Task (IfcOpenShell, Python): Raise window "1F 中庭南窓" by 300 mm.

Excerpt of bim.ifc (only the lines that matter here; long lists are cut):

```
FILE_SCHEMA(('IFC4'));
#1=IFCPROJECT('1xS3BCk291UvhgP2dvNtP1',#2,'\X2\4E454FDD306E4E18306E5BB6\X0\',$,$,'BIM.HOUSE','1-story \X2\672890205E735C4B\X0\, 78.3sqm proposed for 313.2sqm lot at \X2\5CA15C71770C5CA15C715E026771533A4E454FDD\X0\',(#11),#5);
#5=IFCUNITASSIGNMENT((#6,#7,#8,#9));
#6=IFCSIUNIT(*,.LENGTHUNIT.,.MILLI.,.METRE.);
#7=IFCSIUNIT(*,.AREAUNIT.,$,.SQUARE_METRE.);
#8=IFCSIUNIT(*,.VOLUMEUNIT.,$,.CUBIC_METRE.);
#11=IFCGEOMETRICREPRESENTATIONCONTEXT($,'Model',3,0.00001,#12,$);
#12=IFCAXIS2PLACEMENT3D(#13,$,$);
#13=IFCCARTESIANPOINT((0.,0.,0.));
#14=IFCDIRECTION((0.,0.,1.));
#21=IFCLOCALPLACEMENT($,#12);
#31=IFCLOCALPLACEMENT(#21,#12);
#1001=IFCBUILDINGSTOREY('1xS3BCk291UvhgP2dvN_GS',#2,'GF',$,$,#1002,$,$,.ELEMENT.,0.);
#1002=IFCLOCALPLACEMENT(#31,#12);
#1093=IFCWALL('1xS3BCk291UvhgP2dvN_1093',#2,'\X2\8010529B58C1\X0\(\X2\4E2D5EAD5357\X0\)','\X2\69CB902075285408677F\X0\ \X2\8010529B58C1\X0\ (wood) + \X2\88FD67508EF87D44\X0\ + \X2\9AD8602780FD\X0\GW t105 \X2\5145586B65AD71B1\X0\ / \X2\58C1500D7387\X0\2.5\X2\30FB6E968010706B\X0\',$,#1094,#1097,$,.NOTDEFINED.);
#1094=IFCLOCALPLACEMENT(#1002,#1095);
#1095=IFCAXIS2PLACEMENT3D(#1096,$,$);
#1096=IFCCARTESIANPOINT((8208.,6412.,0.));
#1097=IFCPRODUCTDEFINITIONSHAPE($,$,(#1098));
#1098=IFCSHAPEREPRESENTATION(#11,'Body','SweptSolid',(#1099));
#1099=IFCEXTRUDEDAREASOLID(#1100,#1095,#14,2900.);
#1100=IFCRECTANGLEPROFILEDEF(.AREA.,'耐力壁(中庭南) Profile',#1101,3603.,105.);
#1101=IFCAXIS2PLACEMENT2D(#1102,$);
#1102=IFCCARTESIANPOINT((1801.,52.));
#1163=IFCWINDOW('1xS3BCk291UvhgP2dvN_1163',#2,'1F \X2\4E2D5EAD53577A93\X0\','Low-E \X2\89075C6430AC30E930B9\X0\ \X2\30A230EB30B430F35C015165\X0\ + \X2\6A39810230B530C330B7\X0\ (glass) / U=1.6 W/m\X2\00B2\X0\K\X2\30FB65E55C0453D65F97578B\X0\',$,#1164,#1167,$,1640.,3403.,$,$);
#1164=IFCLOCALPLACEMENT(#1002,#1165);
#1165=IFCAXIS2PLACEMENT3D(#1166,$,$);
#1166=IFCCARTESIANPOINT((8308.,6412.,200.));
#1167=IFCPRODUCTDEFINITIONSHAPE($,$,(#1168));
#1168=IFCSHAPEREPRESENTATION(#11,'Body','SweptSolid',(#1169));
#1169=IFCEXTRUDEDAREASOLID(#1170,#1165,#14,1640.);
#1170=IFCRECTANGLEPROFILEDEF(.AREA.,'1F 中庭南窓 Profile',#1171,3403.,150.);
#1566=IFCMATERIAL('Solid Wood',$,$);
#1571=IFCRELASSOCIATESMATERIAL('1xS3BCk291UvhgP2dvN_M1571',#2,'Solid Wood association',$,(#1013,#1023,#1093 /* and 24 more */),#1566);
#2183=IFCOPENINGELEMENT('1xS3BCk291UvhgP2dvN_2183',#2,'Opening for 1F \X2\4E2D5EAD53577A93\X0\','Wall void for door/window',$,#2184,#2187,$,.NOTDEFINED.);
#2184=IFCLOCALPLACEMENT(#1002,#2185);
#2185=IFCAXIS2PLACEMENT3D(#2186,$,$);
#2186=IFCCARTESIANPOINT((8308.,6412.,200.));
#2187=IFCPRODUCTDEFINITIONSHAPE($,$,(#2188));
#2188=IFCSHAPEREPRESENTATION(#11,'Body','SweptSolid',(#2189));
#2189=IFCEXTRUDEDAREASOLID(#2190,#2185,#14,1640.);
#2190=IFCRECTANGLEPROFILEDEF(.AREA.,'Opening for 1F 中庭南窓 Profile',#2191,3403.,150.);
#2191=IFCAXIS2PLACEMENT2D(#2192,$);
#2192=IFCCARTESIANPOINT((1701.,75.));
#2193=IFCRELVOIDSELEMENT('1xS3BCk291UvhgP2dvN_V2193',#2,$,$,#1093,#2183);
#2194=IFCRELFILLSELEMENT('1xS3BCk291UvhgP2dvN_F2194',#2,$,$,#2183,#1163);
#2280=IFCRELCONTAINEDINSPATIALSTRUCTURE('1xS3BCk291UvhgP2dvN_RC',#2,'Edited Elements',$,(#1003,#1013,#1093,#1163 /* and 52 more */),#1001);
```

```python
import numpy as np
import ifcopenshell
import ifcopenshell.api.geometry
import ifcopenshell.util.placement
import ifcopenshell.util.unit

model = ifcopenshell.open("bim.ifc")
unit_scale = ifcopenshell.util.unit.calculate_unit_scale(model)

window = model.by_guid("1xS3BCk291UvhgP2dvN_1163")
opening = window.FillsVoids[0].RelatingOpeningElement
dz = 300.0

shift = np.array([0.0, 0.0, dz])
# The window is not placed relative to its opening, so move both.
for product in (opening, window):
    matrix = ifcopenshell.util.placement.get_local_placement(product.ObjectPlacement)
    matrix[:3, 3] += shift
    ifcopenshell.api.geometry.edit_object_placement(model, product=product, matrix=matrix, is_si=False)

print(f"moved by {dz * unit_scale:+.3f} m")

model.write("bim_rev.ifc")
```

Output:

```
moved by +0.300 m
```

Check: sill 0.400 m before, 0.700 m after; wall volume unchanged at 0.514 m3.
